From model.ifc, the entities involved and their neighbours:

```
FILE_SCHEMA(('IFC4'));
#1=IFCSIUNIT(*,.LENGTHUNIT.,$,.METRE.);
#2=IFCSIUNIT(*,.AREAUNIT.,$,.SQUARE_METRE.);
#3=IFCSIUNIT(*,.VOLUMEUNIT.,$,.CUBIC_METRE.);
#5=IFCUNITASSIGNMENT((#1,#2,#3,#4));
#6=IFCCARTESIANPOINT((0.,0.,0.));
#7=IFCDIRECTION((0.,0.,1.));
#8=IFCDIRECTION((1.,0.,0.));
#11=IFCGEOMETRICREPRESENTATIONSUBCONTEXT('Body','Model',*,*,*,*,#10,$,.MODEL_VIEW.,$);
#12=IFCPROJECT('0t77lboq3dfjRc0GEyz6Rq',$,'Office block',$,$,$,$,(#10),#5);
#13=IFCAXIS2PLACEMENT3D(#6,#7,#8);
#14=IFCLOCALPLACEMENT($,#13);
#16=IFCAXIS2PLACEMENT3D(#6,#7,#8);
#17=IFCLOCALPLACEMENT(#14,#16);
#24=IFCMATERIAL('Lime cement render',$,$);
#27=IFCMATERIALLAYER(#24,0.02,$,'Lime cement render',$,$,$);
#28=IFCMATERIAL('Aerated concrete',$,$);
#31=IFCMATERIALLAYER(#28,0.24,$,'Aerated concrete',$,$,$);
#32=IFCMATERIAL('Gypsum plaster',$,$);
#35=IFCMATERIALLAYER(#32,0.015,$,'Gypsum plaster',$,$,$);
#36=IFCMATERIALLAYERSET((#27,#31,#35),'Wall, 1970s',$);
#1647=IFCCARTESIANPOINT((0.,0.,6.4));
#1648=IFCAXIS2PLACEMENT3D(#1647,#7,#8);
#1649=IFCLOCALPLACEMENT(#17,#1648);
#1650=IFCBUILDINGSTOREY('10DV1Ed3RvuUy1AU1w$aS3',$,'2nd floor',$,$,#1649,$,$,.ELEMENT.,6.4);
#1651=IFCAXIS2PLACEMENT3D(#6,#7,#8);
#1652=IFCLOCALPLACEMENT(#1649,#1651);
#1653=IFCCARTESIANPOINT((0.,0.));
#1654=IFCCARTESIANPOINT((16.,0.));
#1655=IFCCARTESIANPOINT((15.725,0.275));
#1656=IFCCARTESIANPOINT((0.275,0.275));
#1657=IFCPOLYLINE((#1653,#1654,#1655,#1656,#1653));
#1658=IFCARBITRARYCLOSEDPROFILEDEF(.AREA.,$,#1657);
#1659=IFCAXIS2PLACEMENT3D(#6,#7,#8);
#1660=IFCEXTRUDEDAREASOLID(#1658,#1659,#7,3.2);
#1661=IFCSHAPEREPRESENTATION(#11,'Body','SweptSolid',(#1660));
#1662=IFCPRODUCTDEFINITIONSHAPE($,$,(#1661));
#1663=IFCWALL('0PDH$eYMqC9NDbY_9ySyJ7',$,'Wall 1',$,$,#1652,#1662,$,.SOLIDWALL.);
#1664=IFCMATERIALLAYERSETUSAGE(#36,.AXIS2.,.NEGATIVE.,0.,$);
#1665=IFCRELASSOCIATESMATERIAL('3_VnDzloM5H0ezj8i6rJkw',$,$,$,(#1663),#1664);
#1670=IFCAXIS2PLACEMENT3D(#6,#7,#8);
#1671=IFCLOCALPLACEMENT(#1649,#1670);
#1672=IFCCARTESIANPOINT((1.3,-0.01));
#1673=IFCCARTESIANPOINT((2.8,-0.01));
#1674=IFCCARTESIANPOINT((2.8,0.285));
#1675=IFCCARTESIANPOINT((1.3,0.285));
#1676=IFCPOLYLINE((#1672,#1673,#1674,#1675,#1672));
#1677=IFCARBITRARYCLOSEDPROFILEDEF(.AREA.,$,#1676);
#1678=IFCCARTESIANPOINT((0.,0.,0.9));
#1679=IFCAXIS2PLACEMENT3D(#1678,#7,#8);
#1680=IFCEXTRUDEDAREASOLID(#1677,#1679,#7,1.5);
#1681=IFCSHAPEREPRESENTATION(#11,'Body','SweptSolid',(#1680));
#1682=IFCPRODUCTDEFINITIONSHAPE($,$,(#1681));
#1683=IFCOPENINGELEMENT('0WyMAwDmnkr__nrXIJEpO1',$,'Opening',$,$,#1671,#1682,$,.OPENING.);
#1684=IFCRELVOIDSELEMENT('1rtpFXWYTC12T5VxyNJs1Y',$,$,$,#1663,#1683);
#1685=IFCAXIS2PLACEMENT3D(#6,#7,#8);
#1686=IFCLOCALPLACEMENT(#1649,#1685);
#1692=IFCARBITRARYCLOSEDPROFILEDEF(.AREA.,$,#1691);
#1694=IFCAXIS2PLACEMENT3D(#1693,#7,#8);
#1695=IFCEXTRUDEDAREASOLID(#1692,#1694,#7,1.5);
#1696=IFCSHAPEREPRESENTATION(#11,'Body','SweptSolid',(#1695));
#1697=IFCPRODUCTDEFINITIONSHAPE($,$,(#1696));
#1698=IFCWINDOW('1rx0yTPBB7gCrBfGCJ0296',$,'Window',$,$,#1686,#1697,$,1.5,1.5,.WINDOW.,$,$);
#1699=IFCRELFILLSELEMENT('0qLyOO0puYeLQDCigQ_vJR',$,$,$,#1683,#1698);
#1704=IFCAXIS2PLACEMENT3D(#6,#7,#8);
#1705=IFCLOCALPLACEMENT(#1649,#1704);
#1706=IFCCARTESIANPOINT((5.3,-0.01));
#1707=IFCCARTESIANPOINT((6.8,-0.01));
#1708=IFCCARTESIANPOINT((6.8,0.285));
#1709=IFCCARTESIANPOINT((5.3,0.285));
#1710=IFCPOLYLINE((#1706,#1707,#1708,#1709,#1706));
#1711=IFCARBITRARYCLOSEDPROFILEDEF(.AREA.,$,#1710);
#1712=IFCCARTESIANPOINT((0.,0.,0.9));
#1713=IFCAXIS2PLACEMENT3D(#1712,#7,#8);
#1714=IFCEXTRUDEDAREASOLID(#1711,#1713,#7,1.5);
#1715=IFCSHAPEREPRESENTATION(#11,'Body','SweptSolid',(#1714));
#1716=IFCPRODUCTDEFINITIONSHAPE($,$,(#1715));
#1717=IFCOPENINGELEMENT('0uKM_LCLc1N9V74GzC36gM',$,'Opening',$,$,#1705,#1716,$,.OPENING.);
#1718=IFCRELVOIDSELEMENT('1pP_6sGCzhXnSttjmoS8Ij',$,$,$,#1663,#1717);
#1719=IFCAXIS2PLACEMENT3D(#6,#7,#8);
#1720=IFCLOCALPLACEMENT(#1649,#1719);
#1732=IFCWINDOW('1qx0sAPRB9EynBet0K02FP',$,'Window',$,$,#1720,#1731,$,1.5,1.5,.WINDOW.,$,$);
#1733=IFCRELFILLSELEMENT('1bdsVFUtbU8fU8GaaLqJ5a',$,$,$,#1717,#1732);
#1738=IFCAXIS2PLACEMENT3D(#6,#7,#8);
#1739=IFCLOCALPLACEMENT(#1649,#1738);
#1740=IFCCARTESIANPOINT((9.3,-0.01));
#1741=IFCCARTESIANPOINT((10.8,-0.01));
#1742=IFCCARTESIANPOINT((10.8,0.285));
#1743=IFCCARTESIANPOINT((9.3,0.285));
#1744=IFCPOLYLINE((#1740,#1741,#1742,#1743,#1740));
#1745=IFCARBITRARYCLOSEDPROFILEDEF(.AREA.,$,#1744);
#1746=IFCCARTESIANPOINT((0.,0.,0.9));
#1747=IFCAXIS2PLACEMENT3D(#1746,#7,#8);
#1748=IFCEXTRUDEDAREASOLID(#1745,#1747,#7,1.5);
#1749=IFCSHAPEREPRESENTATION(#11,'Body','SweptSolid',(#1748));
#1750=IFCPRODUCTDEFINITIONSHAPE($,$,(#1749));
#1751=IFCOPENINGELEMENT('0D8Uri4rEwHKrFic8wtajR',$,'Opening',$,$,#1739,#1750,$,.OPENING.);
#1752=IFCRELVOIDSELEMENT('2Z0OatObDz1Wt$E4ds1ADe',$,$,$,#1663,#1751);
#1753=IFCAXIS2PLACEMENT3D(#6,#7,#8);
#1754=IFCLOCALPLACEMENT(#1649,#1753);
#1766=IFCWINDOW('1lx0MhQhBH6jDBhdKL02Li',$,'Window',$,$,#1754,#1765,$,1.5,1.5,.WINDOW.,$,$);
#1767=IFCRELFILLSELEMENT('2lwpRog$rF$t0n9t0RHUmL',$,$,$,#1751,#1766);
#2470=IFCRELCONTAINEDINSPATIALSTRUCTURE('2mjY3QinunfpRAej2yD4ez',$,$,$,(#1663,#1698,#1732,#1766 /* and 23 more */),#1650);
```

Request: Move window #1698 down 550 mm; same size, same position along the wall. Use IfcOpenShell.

```python
import numpy as np
import ifcopenshell
import ifcopenshell.api.geometry
import ifcopenshell.util.placement
import ifcopenshell.util.unit

model = ifcopenshell.open("model.ifc")
unit_scale = ifcopenshell.util.unit.calculate_unit_scale(model)

window = model.by_guid("1rx0yTPBB7gCrBfGCJ0296")
opening = window.FillsVoids[0].RelatingOpeningElement
dz = -0.55 / unit_scale

shift = np.array([0.0, 0.0, dz])
# The window is not placed relative to its opening, so move both.
for product in (opening, window):
    matrix = ifcopenshell.util.placement.get_local_placement(product.ObjectPlacement)
    matrix[:3, 3] += shift
    ifcopenshell.api.geometry.edit_object_placement(model, product=product, matrix=matrix, is_si=False)

print(f"moved by {dz * unit_scale:+.3f} m")

model.write("model_updated.ifc")
```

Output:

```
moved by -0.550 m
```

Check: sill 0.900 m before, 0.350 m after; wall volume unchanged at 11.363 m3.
